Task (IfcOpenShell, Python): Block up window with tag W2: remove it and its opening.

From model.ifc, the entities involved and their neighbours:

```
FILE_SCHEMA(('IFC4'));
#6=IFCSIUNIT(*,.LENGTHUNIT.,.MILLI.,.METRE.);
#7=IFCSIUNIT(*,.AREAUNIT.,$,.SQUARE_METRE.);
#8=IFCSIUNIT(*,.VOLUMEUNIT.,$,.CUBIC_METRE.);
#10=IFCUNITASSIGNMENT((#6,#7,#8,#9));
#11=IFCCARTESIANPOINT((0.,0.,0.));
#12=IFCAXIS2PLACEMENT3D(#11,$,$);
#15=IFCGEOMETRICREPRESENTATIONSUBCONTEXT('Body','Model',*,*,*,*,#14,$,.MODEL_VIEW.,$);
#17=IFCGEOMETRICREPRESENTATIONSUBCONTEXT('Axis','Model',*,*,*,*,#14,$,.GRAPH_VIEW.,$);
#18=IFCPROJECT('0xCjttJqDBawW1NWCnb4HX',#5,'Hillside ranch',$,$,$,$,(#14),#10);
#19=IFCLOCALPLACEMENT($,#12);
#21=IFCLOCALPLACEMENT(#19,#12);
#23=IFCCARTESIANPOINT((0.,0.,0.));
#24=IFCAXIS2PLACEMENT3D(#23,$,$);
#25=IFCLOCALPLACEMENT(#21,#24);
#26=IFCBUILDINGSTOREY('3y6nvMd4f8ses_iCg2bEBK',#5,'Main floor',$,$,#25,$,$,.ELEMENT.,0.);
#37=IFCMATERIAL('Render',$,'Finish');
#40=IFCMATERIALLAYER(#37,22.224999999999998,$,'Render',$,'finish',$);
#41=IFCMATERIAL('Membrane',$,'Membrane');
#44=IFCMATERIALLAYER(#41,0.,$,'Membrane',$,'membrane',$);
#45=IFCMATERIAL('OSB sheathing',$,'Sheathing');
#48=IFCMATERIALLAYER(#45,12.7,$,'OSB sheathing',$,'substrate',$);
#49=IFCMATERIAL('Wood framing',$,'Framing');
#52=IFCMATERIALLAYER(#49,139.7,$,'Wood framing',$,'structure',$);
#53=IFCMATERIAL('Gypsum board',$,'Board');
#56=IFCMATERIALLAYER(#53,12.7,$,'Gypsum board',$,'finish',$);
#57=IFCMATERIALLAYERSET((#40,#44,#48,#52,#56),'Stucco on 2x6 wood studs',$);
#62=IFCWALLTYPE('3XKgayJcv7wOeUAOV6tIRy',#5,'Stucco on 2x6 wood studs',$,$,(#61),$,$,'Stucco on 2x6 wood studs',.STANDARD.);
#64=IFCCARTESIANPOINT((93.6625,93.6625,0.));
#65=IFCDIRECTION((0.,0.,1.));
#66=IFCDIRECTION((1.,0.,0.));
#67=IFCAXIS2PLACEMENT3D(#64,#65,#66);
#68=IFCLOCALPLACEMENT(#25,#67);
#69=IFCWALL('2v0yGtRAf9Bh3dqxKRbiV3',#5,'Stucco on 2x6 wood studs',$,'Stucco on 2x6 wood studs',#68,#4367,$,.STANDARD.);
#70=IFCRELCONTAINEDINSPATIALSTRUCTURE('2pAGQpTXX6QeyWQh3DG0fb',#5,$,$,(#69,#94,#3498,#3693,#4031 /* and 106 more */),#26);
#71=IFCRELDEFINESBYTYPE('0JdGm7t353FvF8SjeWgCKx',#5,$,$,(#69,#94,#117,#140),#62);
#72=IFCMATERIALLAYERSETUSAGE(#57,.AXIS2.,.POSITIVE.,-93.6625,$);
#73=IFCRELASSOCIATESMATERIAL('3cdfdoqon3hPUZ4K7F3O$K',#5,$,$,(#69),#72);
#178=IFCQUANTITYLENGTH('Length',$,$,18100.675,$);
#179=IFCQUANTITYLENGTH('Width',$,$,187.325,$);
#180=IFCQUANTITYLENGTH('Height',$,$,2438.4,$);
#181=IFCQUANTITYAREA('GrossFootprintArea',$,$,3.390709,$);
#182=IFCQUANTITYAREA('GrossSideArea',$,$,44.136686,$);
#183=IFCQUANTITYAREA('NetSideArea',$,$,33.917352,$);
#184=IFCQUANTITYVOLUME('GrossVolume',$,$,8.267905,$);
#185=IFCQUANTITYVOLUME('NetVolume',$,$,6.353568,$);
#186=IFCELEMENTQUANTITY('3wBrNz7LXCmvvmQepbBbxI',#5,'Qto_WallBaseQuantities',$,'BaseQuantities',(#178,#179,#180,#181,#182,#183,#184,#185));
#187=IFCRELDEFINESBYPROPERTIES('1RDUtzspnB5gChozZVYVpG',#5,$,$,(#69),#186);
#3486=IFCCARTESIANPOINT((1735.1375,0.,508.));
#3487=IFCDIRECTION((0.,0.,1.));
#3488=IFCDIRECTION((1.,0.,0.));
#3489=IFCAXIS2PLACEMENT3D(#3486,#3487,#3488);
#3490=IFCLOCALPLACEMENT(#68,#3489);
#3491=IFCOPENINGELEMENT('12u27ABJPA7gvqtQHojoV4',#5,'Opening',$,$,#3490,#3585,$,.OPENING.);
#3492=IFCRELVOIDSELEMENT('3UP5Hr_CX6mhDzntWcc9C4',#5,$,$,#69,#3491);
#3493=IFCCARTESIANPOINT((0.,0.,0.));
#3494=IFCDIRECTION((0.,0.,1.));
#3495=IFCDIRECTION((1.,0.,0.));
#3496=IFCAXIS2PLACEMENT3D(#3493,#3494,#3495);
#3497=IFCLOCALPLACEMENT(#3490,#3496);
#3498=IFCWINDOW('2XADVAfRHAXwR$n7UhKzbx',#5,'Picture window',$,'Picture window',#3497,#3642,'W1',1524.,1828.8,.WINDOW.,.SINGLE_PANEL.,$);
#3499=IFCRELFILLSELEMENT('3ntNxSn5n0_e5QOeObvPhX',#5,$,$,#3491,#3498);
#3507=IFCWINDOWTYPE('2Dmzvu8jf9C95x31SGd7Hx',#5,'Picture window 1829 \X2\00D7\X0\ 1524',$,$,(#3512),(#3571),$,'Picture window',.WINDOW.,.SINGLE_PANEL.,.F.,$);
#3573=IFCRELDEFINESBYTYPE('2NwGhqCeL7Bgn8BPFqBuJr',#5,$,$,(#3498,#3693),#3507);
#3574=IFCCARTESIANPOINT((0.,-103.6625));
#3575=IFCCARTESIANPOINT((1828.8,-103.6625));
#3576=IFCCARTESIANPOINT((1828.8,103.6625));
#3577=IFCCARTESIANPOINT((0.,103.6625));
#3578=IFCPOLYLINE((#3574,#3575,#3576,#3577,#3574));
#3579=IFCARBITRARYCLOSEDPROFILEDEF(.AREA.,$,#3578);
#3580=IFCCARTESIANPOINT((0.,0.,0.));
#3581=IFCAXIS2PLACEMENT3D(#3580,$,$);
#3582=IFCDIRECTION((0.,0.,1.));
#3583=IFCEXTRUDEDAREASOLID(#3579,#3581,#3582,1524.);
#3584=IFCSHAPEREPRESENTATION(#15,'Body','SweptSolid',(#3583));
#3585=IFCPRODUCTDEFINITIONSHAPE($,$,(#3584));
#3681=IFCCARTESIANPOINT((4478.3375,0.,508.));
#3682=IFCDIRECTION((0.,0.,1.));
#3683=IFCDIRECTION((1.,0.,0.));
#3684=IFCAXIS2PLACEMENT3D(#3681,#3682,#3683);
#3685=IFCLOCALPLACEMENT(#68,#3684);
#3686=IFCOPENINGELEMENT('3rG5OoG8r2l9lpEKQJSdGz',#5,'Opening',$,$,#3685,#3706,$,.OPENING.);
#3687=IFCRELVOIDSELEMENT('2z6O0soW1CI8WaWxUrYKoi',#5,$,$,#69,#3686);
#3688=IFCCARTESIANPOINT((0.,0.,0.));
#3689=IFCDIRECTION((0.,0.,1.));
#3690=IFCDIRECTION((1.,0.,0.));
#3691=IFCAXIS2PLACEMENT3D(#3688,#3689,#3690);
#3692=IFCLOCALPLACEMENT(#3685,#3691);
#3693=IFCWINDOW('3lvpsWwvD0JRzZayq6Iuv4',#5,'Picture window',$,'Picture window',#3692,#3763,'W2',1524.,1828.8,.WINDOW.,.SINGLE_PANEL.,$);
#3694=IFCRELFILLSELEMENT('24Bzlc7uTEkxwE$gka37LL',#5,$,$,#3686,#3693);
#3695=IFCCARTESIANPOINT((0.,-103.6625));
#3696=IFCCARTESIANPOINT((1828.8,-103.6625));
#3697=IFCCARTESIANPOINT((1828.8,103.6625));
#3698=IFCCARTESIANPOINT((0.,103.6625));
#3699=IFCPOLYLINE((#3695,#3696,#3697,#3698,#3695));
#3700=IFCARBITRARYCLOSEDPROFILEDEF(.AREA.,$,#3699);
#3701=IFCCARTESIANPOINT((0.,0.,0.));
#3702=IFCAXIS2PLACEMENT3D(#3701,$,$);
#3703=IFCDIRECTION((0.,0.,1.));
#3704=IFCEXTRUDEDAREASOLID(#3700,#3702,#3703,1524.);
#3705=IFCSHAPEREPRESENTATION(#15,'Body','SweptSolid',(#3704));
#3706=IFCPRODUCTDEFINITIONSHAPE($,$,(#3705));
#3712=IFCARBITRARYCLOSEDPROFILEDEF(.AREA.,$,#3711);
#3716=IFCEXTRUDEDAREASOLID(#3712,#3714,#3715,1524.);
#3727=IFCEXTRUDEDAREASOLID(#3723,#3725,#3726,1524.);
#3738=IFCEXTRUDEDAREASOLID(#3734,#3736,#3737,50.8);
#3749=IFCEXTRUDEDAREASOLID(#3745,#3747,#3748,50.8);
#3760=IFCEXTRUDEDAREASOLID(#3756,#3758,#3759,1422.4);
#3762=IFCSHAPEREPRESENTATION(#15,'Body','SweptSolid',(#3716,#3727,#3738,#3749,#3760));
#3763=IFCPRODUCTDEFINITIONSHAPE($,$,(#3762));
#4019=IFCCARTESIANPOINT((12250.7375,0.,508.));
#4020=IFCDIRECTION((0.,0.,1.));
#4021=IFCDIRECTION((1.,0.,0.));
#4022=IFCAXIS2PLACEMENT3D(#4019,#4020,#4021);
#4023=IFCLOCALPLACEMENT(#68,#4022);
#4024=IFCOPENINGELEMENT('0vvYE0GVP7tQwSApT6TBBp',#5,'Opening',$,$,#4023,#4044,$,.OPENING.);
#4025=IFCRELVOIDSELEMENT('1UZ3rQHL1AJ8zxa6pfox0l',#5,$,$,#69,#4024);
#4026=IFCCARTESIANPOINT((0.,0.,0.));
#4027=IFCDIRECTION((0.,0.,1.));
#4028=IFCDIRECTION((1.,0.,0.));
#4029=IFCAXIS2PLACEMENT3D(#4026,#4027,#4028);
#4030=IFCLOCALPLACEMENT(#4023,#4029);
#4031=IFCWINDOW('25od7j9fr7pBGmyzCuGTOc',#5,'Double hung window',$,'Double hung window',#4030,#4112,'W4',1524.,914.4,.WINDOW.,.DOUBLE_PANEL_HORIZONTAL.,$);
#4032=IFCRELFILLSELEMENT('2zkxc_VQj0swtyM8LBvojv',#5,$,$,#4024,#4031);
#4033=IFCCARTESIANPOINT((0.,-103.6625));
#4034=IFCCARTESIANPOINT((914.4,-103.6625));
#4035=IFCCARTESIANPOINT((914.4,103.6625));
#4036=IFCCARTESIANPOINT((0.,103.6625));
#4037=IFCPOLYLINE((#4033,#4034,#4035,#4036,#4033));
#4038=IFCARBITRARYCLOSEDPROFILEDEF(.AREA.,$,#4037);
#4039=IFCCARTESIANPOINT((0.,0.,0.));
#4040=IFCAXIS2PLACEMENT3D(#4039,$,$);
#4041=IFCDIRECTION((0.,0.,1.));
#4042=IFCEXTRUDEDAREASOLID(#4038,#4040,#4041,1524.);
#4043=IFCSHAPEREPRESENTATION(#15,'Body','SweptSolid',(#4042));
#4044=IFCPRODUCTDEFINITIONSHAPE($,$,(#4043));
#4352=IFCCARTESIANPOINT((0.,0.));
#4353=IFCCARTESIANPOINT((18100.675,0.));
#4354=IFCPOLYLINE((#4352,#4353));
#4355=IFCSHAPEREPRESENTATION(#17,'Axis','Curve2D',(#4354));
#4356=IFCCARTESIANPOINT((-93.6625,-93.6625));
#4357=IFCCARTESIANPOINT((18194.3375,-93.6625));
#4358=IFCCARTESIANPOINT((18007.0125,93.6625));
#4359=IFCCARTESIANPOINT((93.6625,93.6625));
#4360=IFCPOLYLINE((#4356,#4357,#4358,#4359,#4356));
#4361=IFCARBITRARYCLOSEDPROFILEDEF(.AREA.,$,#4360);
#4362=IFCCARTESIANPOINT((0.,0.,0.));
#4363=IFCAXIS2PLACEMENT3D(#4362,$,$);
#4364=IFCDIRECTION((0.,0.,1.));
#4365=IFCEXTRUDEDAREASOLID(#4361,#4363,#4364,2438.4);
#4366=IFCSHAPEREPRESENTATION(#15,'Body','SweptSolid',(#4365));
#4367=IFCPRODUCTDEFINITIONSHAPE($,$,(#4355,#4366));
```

```python
import ifcopenshell
import ifcopenshell.api.feature
import ifcopenshell.api.pset
import ifcopenshell.api.root
import ifcopenshell.geom
import ifcopenshell.util.element
import ifcopenshell.util.shape
import ifcopenshell.util.unit

model = ifcopenshell.open("model.ifc")
area_scale = ifcopenshell.util.unit.calculate_unit_scale(model, "AREAUNIT")
volume_scale = ifcopenshell.util.unit.calculate_unit_scale(model, "VOLUMEUNIT")
settings = ifcopenshell.geom.settings()


def volume(element):
    """Net volume in cubic metres, openings subtracted."""
    shape = ifcopenshell.geom.create_shape(settings, element)
    return ifcopenshell.util.shape.get_volume(shape.geometry)


window = model.by_id(3693)
opening = window.FillsVoids[0].RelatingOpeningElement
wall = opening.VoidsElements[0].RelatingBuildingElement
before = volume(wall)

ifcopenshell.api.root.remove_product(model, product=window)
ifcopenshell.api.feature.remove_feature(model, feature=opening)

after = volume(wall)
thickness = 0.1873  # wall thickness in metres

# Update the wall's stored quantities.
qto = model.by_id(ifcopenshell.util.element.get_pset(wall, "Qto_WallBaseQuantities", should_inherit=False)["id"])
ifcopenshell.api.pset.edit_qto(model, qto=qto, properties={
    "NetSideArea": after / thickness / area_scale,
    "NetVolume": after / volume_scale,
})

print(f"wall volume {before:.3f} -> {after:.3f} m3")

model.write("model_updated.ifc")
```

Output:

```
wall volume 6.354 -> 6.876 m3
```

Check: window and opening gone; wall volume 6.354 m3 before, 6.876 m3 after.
